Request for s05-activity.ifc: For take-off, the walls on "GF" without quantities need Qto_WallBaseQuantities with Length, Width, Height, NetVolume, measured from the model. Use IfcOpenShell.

First a look at what the model holds.

```python
import ifcopenshell
import ifcopenshell.util.element
import ifcopenshell.util.unit

model = ifcopenshell.open("s05-activity.ifc")
print(model.schema)
for unit_type in ("LENGTHUNIT", "AREAUNIT", "VOLUMEUNIT"):
    print(unit_type, ifcopenshell.util.unit.calculate_unit_scale(model, unit_type))
storey = next(s for s in model.by_type("IfcBuildingStorey") if s.Name == "GF")
walls = [e for e in ifcopenshell.util.element.get_decomposition(storey) if e.is_a("IfcWall")]
for e in sorted(walls, key=lambda e: e.id()):
    print(e.id(), e.is_a(), e.Name, list(ifcopenshell.util.element.get_psets(e, qtos_only=True)), sep=" | ")
```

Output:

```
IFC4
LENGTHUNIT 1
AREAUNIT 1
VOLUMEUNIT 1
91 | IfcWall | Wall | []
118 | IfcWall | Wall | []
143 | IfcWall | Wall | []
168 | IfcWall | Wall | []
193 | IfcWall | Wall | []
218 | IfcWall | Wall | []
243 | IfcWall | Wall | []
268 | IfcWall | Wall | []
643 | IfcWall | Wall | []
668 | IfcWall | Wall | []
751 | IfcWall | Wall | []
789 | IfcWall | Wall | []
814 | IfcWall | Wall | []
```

```python
import ifcopenshell
import ifcopenshell.api.pset
import ifcopenshell.geom
import ifcopenshell.util.element
import ifcopenshell.util.shape
import ifcopenshell.util.unit

model = ifcopenshell.open("s05-activity.ifc")
unit_scale = ifcopenshell.util.unit.calculate_unit_scale(model)
volume_scale = ifcopenshell.util.unit.calculate_unit_scale(model, "VOLUMEUNIT")
settings = ifcopenshell.geom.settings()

storey = next(s for s in model.by_type("IfcBuildingStorey") if s.Name == "GF")
walls = [e for e in ifcopenshell.util.element.get_decomposition(storey) if e.is_a("IfcWall")]

for e in sorted(walls, key=lambda e: e.id()):
    if ifcopenshell.util.element.get_psets(e, qtos_only=True, should_inherit=False):
        continue
    # Geometry comes back in metres, in the element's own axes.
    shape = ifcopenshell.geom.create_shape(settings, e)
    values = {
        "Length": ifcopenshell.util.shape.get_x(shape.geometry) / unit_scale,
        "Width": ifcopenshell.util.shape.get_y(shape.geometry) / unit_scale,
        "Height": ifcopenshell.util.shape.get_z(shape.geometry) / unit_scale,
        "NetVolume": ifcopenshell.util.shape.get_volume(shape.geometry) / volume_scale,
    }
    qto = ifcopenshell.api.pset.add_qto(model, product=e, name="Qto_WallBaseQuantities")
    ifcopenshell.api.pset.edit_qto(model, qto=qto, properties=values)
    print(e.id(), {k: round(v, 3) for k, v in values.items()})

model.write("s05-activity-out.ifc")
```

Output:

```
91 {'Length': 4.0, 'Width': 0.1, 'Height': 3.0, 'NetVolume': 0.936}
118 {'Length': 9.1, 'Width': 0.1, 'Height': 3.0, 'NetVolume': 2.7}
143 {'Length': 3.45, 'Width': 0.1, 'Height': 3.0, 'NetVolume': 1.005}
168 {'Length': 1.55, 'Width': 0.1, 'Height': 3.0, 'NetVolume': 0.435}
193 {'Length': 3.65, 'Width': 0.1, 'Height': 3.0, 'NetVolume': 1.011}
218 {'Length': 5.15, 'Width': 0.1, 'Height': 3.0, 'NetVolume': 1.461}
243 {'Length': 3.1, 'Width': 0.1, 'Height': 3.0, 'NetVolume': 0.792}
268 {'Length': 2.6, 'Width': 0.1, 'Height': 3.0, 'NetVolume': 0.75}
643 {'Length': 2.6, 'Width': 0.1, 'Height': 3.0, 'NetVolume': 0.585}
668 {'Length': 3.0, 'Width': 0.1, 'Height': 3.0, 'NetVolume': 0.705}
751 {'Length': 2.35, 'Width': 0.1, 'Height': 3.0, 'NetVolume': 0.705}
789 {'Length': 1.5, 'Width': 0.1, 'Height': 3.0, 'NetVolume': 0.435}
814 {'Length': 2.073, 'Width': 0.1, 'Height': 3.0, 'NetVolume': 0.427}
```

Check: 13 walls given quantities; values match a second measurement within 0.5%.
